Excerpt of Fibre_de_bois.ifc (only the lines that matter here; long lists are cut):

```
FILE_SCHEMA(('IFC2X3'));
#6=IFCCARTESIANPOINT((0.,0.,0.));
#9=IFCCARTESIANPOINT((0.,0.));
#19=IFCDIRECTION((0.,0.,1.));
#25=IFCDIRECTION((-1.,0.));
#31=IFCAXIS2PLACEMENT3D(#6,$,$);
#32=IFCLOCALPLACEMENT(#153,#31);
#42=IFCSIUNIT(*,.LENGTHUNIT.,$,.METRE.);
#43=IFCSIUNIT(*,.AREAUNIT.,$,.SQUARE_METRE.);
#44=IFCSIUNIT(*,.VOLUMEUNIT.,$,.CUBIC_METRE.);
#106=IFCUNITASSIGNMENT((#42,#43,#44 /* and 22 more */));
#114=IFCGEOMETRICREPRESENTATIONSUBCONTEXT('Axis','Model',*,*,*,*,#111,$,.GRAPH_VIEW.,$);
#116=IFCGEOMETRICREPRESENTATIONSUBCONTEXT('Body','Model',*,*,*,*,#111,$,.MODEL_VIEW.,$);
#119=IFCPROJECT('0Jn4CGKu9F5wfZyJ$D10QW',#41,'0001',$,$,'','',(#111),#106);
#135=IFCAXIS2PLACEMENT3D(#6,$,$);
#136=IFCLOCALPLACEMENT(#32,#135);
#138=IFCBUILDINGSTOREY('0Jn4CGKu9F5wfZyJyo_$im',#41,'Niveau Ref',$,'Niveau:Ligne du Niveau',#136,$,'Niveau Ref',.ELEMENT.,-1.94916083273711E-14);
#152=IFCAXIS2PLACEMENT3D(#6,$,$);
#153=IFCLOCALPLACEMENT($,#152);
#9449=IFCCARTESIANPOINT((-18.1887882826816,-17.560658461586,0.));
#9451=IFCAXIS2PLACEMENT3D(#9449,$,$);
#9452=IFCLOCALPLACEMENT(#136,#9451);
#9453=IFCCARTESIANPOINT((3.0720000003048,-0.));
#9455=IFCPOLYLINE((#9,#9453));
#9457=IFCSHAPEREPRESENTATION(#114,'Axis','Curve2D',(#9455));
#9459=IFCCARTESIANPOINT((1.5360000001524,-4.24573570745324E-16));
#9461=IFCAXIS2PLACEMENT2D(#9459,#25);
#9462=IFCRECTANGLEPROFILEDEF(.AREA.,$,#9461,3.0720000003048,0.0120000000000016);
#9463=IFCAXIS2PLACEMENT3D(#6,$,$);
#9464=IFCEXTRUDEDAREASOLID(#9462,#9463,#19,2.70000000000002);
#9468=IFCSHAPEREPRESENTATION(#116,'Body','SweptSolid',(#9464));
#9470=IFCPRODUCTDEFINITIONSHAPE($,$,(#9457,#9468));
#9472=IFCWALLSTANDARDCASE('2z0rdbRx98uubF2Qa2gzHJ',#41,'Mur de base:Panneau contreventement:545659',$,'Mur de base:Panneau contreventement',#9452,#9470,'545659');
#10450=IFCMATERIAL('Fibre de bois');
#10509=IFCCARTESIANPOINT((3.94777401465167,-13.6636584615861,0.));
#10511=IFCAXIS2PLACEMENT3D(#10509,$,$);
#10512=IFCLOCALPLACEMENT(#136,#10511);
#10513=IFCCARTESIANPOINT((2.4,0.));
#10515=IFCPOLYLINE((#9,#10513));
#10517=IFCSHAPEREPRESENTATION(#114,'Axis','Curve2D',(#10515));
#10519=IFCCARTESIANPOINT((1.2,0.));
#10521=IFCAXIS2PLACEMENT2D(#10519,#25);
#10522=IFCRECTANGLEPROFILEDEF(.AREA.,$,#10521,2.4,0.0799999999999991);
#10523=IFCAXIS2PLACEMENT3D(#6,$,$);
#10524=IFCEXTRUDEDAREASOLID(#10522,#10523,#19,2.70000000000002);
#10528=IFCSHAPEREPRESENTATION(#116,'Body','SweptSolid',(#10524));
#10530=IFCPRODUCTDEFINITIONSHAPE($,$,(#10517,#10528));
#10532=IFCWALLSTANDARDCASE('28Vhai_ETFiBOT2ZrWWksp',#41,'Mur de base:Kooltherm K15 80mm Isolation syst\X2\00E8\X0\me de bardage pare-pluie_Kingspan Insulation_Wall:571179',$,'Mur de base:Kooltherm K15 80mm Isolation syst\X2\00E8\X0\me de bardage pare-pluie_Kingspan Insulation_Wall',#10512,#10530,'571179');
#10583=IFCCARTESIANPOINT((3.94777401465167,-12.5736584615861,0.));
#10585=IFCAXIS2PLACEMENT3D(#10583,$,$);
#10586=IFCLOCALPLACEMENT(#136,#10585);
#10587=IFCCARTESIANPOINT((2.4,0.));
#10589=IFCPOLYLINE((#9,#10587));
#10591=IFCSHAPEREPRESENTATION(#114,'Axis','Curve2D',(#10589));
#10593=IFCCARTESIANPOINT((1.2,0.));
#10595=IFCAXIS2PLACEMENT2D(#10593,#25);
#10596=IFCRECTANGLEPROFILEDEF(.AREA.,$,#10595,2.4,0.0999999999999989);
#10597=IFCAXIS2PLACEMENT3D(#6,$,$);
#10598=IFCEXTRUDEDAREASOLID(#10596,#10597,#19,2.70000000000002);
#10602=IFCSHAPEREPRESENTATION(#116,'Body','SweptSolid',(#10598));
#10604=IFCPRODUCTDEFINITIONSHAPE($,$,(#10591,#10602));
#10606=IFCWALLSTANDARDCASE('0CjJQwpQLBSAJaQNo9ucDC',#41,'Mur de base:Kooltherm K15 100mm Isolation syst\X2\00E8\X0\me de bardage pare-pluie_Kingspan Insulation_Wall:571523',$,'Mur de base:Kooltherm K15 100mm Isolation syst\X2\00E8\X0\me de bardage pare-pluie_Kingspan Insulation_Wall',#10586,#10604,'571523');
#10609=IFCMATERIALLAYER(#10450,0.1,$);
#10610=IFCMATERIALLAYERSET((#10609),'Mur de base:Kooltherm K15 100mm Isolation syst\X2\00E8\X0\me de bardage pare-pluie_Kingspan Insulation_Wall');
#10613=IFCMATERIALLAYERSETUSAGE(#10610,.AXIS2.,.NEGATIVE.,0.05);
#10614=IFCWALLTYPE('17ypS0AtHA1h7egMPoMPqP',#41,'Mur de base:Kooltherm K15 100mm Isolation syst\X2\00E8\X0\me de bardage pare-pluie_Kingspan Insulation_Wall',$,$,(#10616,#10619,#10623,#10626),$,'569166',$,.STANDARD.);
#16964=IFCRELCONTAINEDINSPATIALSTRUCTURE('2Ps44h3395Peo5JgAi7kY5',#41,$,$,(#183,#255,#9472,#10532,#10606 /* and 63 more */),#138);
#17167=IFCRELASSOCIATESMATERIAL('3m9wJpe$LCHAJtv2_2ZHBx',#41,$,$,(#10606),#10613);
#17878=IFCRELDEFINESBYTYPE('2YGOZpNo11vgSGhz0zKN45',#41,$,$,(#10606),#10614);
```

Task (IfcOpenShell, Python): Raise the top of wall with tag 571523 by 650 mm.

```python
import ifcopenshell
import ifcopenshell.geom
import ifcopenshell.util.representation
import ifcopenshell.util.shape

model = ifcopenshell.open("Fibre_de_bois.ifc")
settings = ifcopenshell.geom.settings()


def volume(element):
    """Net volume in cubic metres, openings subtracted."""
    shape = ifcopenshell.geom.create_shape(settings, element)
    return ifcopenshell.util.shape.get_volume(shape.geometry)


wall = model.by_id(10606)
before = volume(wall)

body = ifcopenshell.util.representation.get_representation(wall, "Model", "Body")
solid = body.Items[0]
old_height = solid.Depth
solid.Depth += 0.65
after = volume(wall)

print(f"height {old_height:g} -> {solid.Depth:g}, volume {before:.3f} -> {after:.3f} m3")

model.write("Fibre_de_bois_rev.ifc")
```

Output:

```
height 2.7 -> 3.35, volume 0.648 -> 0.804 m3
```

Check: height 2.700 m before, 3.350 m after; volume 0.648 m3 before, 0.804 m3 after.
